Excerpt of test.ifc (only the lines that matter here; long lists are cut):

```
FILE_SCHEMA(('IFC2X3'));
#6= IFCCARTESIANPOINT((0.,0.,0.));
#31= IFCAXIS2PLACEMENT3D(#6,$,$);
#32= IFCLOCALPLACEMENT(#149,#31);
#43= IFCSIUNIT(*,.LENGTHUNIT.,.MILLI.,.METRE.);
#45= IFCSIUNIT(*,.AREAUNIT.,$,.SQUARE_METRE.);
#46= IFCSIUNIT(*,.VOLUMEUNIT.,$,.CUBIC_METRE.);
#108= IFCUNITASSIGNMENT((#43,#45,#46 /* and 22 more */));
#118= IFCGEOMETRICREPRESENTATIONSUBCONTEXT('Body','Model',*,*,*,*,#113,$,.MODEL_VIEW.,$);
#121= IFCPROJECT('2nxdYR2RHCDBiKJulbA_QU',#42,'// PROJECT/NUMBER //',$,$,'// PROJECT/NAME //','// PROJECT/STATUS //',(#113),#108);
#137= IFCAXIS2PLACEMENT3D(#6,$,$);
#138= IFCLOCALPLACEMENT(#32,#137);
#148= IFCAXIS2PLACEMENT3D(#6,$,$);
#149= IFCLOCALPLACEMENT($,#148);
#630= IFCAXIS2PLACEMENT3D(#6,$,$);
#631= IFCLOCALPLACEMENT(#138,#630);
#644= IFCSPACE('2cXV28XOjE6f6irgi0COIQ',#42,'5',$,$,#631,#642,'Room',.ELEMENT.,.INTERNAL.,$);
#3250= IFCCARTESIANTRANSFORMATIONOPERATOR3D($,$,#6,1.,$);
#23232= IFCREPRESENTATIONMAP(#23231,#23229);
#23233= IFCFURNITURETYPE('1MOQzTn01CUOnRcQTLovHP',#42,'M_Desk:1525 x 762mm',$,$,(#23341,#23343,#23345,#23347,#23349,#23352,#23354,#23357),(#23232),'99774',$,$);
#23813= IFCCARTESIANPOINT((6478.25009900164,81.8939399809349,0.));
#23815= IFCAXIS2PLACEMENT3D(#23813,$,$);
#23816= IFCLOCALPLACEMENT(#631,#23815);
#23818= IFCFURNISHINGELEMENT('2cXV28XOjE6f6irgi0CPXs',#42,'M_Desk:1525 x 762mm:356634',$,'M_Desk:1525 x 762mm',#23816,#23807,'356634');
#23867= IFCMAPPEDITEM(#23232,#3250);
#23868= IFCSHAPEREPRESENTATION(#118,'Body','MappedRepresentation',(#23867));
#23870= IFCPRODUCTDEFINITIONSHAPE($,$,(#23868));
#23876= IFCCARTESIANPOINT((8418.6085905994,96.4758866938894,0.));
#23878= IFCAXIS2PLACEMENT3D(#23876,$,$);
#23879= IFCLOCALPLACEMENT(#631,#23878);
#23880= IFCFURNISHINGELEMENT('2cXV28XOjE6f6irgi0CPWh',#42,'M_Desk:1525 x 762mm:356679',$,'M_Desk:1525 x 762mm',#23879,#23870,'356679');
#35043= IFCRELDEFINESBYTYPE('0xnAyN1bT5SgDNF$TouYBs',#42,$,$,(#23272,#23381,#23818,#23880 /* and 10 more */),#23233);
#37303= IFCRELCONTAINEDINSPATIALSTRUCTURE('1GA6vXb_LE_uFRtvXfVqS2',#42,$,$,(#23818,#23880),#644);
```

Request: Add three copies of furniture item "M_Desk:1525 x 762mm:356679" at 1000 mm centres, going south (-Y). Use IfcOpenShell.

```python
import numpy as np
import ifcopenshell
import ifcopenshell.api.geometry
import ifcopenshell.api.root
import ifcopenshell.util.element
import ifcopenshell.util.placement

model = ifcopenshell.open("test.ifc")


def reuse_history(source, copy):
    """copy_class also copies each property set's owner history, people and application; keep the originals."""
    for rel in copy.IsDefinedBy:
        if rel.is_a("IfcRelDefinesByProperties") and (history := rel.RelatingPropertyDefinition.OwnerHistory):
            rel.RelatingPropertyDefinition.OwnerHistory = source.OwnerHistory
            ifcopenshell.util.element.remove_deep2(model, history)


source = model.by_id(23880)
base = ifcopenshell.util.placement.get_local_placement(source.ObjectPlacement)
step = np.array([0.0, -1.0, 0.0]) * 1000.0

for i in range(1, 4):
    copy = ifcopenshell.api.root.copy_class(model, product=source)
    copy.Representation = ifcopenshell.util.element.copy_deep(
        model, source.Representation, exclude=["IfcGeometricRepresentationContext", "IfcRepresentationMap"]
    )
    copy.Name = "M_Desk:1525 x 762mm"
    copy.Tag = None
    reuse_history(source, copy)
    matrix = base.copy()
    matrix[:3, 3] += i * step
    print("added at", matrix[:3, 3].round(3) + 0.0)
    ifcopenshell.api.geometry.edit_object_placement(model, product=copy, matrix=matrix, is_si=False)

model.write("test_edited.ifc")
```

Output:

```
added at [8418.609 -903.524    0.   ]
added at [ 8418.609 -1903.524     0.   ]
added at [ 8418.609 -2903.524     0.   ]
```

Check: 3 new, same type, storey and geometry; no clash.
